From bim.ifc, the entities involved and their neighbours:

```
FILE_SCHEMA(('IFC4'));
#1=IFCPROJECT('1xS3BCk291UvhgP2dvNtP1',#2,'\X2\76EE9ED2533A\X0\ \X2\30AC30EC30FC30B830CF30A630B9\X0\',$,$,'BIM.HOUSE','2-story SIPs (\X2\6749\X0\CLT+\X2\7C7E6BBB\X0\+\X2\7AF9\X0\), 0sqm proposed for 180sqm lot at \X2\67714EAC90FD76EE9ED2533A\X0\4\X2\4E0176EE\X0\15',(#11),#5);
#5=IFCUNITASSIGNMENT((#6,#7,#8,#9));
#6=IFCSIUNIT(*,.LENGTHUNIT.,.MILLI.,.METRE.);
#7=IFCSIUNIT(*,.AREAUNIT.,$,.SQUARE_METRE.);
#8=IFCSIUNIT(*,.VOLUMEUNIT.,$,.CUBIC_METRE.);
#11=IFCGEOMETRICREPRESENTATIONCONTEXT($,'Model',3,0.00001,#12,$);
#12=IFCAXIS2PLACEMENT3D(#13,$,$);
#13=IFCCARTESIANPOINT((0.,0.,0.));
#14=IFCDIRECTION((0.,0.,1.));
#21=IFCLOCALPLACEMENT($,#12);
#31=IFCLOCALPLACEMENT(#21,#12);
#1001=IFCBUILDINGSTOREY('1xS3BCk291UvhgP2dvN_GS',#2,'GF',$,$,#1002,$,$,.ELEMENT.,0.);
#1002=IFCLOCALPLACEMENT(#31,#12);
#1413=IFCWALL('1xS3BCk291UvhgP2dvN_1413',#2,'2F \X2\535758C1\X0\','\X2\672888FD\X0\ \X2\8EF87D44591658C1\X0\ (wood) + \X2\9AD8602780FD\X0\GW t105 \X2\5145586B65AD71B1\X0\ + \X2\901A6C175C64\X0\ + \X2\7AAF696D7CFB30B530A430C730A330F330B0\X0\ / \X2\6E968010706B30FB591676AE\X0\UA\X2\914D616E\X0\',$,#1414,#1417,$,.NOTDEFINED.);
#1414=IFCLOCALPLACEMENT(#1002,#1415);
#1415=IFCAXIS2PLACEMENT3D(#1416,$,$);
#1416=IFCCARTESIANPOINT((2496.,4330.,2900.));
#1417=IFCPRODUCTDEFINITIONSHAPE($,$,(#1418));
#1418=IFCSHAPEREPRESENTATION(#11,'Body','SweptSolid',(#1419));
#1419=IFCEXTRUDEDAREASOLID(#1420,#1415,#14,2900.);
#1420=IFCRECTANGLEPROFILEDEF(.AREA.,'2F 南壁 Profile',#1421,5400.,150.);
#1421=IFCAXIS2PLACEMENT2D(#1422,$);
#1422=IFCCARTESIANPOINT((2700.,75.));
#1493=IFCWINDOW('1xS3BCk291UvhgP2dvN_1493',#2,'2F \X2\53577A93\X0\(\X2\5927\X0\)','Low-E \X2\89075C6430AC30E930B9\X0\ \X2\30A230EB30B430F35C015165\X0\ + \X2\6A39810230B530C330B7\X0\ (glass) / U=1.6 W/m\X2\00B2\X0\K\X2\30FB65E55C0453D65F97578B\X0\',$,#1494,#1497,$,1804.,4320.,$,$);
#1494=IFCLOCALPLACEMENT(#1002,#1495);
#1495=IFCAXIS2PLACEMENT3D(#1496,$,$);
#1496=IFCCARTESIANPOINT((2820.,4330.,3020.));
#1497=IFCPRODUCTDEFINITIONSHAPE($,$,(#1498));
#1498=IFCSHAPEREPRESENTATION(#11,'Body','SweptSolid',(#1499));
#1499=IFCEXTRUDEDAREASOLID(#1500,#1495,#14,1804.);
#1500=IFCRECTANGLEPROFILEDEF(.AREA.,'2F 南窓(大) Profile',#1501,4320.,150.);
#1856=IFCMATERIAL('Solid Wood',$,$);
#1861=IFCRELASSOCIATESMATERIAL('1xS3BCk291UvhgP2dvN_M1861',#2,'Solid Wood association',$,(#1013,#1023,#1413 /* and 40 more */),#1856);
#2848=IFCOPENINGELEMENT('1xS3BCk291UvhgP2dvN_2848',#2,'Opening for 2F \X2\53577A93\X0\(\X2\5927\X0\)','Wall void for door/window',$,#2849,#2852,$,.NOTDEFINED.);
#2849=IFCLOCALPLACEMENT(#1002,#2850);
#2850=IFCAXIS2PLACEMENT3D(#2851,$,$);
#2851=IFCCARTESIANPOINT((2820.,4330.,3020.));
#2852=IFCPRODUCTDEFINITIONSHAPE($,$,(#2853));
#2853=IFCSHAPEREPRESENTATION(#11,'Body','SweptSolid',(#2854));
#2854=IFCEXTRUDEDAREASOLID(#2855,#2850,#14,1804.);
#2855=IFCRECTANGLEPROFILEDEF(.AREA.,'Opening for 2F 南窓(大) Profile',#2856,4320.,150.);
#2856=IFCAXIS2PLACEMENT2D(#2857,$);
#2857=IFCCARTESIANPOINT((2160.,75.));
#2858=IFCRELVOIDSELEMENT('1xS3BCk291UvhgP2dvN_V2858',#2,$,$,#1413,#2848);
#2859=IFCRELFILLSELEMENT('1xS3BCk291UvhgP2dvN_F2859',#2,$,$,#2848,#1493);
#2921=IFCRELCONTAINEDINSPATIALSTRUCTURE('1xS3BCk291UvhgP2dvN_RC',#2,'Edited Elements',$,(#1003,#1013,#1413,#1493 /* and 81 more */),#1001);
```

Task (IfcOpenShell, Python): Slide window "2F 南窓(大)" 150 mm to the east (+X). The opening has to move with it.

```python
import ifcopenshell
import ifcopenshell.api.geometry
import ifcopenshell.util.placement
import ifcopenshell.util.unit

model = ifcopenshell.open("bim.ifc")
unit_scale = ifcopenshell.util.unit.calculate_unit_scale(model)

window = model.by_guid("1xS3BCk291UvhgP2dvN_1493")
opening = window.FillsVoids[0].RelatingOpeningElement
wall = opening.VoidsElements[0].RelatingBuildingElement

wall_matrix = ifcopenshell.util.placement.get_local_placement(wall.ObjectPlacement)
shift = wall_matrix[:3, 0] * 0.15 / unit_scale
before = ifcopenshell.util.placement.get_local_placement(window.ObjectPlacement)[:3, 3].copy()

# The window is not placed relative to its opening, so move both.
for product in (opening, window):
    matrix = ifcopenshell.util.placement.get_local_placement(product.ObjectPlacement)
    matrix[:3, 3] += shift
    ifcopenshell.api.geometry.edit_object_placement(model, product=product, matrix=matrix, is_si=False)

after = ifcopenshell.util.placement.get_local_placement(window.ObjectPlacement)[:3, 3]
print("window moved by", (after - before).round(3) + 0.0)

model.write("bim_rev.ifc")
```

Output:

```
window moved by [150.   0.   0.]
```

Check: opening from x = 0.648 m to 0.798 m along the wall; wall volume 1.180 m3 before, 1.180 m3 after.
